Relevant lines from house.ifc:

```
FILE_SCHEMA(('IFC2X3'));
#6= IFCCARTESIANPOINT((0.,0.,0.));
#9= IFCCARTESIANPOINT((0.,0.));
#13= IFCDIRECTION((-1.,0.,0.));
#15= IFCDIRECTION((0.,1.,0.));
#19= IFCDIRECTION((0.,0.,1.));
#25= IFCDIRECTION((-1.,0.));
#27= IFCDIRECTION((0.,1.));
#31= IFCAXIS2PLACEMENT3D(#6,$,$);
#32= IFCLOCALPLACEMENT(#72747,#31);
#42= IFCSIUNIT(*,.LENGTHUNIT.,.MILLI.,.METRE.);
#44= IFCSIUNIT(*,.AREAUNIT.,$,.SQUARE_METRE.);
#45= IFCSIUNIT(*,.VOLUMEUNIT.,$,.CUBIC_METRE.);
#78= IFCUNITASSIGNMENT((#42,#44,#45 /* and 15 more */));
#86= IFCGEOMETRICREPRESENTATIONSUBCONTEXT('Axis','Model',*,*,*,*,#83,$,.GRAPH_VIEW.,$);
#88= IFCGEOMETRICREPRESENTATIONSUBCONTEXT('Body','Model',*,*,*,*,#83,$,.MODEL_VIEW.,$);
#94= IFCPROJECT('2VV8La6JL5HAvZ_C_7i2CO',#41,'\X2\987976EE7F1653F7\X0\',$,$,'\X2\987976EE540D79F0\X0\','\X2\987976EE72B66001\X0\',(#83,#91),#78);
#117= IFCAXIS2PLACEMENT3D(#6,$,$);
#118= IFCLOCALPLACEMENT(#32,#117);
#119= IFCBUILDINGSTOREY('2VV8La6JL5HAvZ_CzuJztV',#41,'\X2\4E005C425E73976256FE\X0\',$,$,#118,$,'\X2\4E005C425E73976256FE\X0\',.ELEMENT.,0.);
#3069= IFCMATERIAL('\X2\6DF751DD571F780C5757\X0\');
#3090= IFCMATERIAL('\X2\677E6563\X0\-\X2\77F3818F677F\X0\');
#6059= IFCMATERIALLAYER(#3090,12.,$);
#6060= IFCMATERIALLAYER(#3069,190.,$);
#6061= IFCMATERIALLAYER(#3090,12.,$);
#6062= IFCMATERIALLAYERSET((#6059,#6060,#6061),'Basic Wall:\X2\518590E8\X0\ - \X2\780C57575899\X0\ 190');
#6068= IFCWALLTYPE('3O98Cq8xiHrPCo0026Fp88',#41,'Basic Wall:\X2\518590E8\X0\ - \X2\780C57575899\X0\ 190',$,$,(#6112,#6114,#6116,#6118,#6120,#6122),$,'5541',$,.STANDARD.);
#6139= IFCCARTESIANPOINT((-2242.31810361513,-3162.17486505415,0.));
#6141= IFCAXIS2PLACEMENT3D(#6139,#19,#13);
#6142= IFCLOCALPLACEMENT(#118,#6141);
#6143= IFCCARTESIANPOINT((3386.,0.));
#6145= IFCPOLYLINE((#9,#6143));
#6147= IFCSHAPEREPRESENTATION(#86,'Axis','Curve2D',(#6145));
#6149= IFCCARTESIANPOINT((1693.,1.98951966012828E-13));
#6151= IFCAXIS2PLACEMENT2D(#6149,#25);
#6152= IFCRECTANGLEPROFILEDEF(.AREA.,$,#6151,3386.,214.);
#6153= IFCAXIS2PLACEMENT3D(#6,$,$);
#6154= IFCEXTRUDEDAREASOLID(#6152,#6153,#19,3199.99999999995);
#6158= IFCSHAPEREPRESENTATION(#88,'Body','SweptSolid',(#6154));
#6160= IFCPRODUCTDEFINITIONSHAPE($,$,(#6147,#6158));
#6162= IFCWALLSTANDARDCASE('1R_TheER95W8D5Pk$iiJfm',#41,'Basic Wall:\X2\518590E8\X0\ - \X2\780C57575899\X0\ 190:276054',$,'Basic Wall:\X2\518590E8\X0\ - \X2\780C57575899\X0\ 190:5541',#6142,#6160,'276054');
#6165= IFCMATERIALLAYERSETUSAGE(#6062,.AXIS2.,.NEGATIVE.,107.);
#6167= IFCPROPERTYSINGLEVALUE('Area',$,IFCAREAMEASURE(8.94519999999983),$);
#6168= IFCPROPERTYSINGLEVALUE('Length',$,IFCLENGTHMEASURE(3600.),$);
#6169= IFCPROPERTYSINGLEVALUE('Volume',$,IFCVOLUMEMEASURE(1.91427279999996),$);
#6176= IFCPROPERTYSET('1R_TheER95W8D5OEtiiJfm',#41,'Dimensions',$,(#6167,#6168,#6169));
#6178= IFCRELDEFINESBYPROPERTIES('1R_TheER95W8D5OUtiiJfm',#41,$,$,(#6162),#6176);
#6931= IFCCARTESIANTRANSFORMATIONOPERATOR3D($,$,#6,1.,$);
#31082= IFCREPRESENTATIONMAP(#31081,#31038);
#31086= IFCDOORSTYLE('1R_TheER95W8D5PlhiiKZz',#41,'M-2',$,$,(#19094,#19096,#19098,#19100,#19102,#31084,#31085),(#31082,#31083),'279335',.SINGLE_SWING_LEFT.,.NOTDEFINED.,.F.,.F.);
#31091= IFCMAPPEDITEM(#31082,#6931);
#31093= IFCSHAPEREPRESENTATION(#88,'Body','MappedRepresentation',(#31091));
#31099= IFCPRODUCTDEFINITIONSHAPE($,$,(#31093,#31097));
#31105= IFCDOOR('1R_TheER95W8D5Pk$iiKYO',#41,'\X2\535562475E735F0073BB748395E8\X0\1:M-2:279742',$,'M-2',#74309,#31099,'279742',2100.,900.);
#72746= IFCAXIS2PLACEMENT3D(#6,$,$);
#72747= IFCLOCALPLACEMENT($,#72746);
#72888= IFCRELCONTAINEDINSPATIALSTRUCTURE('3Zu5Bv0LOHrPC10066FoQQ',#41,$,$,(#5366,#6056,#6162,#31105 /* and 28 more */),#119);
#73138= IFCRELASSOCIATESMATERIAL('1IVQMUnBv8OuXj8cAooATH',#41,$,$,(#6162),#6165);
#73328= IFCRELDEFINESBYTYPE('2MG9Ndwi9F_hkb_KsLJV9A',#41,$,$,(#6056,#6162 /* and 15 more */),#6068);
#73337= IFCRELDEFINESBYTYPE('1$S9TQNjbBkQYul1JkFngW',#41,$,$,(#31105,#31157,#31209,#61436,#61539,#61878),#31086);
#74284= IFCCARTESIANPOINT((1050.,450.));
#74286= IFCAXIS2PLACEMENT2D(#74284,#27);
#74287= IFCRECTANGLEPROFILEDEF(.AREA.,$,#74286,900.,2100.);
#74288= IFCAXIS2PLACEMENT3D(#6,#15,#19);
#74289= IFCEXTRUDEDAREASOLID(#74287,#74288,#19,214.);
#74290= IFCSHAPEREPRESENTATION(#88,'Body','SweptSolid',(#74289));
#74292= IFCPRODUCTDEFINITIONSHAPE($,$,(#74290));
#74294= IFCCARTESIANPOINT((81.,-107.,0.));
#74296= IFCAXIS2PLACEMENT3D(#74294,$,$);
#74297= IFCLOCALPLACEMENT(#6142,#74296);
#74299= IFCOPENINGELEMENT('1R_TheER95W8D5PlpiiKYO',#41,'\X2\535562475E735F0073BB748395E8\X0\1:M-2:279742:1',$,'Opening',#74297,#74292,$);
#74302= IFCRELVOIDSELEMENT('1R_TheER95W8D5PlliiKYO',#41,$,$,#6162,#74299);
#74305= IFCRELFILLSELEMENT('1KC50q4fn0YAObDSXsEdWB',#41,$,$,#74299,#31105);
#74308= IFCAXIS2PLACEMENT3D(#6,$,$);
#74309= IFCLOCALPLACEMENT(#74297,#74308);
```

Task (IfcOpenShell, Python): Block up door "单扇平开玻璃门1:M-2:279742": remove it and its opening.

```python
import ifcopenshell
import ifcopenshell.api.feature
import ifcopenshell.api.pset
import ifcopenshell.api.root
import ifcopenshell.geom
import ifcopenshell.util.element
import ifcopenshell.util.shape
import ifcopenshell.util.unit

model = ifcopenshell.open("house.ifc")
area_scale = ifcopenshell.util.unit.calculate_unit_scale(model, "AREAUNIT")
volume_scale = ifcopenshell.util.unit.calculate_unit_scale(model, "VOLUMEUNIT")
settings = ifcopenshell.geom.settings()


def volume(element):
    """Net volume in cubic metres, openings subtracted."""
    shape = ifcopenshell.geom.create_shape(settings, element)
    return ifcopenshell.util.shape.get_volume(shape.geometry)


door = model.by_id(31105)
opening = door.FillsVoids[0].RelatingOpeningElement
wall = opening.VoidsElements[0].RelatingBuildingElement
before = volume(wall)

ifcopenshell.api.root.remove_product(model, product=door)
ifcopenshell.api.feature.remove_feature(model, feature=opening)

after = volume(wall)
thickness = 0.214  # wall thickness in metres

# Update the wall's stored quantities.
pset = model.by_id(ifcopenshell.util.element.get_pset(wall, "Dimensions", should_inherit=False)["id"])
ifcopenshell.api.pset.edit_pset(model, pset=pset, properties={
    "Area": model.create_entity("IfcAreaMeasure", after / thickness / area_scale),
    "Volume": model.create_entity("IfcVolumeMeasure", after / volume_scale),
})

print(f"wall volume {before:.3f} -> {after:.3f} m3")

model.write("house_updated.ifc")
```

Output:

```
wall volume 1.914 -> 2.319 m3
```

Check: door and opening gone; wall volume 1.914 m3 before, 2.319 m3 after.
